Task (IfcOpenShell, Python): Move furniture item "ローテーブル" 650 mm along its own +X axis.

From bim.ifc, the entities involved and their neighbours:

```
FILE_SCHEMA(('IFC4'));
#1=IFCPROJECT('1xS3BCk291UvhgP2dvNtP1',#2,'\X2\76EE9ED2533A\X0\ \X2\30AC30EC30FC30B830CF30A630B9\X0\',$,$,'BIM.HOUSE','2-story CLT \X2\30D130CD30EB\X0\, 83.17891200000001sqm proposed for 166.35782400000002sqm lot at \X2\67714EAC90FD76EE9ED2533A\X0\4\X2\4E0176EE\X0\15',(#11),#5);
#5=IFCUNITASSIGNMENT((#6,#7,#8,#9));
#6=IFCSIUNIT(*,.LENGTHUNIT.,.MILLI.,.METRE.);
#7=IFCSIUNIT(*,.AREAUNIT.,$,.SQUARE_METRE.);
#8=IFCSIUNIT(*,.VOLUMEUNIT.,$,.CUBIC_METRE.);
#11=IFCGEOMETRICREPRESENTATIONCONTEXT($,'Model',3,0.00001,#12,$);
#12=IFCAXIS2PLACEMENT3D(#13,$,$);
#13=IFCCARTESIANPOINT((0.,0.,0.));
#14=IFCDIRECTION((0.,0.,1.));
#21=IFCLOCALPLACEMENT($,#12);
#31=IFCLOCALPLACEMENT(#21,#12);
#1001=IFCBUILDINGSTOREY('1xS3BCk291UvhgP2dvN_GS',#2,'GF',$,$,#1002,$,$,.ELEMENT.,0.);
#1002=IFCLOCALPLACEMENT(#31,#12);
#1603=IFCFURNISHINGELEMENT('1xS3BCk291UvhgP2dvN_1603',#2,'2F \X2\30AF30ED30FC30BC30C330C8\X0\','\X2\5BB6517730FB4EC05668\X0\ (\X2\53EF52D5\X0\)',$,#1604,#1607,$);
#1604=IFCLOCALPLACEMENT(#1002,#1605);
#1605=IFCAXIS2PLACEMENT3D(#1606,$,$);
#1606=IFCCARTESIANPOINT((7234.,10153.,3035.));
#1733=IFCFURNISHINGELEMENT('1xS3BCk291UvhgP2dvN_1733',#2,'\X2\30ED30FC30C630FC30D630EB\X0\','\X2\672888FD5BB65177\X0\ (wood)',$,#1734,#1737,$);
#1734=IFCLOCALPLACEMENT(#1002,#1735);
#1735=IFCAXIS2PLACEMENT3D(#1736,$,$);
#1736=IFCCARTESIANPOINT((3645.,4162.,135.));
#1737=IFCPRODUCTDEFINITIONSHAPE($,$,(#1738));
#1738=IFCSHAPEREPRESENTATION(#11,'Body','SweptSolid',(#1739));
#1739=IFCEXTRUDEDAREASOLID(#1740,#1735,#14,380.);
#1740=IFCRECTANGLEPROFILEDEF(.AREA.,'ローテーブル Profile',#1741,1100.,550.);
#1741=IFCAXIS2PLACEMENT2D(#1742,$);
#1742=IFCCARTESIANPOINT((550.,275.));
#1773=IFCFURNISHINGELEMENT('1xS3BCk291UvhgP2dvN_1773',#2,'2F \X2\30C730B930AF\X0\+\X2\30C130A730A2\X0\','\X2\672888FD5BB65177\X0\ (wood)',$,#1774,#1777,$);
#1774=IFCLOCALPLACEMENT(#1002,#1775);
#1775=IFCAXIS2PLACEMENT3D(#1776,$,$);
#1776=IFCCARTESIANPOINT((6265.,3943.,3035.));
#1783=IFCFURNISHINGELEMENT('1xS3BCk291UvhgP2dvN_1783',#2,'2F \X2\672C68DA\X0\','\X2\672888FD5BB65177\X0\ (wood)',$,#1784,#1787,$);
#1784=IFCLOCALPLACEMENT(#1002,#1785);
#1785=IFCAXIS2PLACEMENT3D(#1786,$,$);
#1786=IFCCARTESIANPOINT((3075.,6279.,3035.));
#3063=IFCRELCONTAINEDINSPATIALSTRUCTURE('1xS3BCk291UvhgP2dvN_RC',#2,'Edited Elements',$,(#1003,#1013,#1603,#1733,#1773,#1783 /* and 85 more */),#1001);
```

```python
import ifcopenshell
import ifcopenshell.api.geometry
import ifcopenshell.util.placement

model = ifcopenshell.open("bim.ifc")

item = model.by_guid("1xS3BCk291UvhgP2dvN_1733")
matrix = ifcopenshell.util.placement.get_local_placement(item.ObjectPlacement)
matrix[:3, 3] += matrix[:3, 0] * 650.0
ifcopenshell.api.geometry.edit_object_placement(model, product=item, matrix=matrix, is_si=False)

print(ifcopenshell.util.placement.get_local_placement(item.ObjectPlacement).round(3) + 0.0)

model.write("bim-out.ifc")
```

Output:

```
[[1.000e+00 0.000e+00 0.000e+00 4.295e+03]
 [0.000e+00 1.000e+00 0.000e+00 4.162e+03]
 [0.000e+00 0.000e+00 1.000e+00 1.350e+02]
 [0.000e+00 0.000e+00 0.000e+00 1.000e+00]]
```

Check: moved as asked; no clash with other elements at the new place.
